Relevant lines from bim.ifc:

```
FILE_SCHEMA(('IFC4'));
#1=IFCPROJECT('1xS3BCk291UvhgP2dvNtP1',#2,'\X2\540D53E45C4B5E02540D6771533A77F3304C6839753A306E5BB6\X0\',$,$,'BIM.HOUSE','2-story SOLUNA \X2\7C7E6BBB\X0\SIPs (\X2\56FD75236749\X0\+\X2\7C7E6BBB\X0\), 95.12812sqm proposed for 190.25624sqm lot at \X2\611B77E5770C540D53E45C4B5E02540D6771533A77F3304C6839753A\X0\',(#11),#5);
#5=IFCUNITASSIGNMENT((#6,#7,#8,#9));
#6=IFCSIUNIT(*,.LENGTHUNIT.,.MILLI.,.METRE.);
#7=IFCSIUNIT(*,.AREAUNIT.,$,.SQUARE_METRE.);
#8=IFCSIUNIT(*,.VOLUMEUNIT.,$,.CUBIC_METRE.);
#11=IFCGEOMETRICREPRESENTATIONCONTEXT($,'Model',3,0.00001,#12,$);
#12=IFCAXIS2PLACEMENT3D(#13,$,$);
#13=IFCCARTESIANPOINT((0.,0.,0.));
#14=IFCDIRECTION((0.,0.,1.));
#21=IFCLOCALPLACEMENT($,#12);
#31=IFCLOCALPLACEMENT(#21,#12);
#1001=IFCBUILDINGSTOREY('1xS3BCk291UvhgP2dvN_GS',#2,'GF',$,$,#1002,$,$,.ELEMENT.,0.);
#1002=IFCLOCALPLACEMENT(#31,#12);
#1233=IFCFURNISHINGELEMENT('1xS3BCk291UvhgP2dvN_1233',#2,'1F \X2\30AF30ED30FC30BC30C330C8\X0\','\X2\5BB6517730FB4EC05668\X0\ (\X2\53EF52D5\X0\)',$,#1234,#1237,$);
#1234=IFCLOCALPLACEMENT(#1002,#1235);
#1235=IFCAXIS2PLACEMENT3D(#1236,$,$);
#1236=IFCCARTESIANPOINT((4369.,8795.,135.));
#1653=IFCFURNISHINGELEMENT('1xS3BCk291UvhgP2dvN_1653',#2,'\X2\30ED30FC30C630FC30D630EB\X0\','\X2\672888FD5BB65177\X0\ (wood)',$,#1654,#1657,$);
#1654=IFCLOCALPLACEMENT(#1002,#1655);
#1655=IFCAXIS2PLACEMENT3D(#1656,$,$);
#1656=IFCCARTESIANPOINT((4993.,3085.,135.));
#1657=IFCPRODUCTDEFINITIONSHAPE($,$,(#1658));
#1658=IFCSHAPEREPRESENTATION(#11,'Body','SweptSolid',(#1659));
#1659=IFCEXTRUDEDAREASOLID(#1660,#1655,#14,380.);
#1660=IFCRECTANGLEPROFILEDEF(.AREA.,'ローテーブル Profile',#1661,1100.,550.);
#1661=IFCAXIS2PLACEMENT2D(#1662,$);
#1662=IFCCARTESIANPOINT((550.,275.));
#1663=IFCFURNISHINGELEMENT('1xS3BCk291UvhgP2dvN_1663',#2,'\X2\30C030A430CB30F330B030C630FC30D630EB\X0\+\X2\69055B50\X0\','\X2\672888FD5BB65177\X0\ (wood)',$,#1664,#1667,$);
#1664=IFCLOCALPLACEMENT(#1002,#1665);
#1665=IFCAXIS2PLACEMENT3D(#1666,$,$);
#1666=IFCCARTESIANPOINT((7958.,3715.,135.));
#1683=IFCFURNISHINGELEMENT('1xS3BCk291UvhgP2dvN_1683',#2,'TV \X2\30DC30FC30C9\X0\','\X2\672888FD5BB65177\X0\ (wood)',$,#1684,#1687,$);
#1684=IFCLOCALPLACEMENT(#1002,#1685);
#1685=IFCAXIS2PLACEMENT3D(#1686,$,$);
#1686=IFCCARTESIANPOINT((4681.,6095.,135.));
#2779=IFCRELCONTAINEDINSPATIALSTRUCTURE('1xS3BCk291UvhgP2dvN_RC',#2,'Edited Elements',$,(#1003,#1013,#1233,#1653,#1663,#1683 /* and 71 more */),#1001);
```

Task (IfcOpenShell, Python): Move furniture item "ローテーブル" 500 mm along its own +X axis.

```python
import ifcopenshell
import ifcopenshell.api.geometry
import ifcopenshell.util.placement
import ifcopenshell.util.unit

model = ifcopenshell.open("bim.ifc")
unit_scale = ifcopenshell.util.unit.calculate_unit_scale(model)

item = model.by_id(1653)
matrix = ifcopenshell.util.placement.get_local_placement(item.ObjectPlacement)
matrix[:3, 3] += matrix[:3, 0] * 0.5 / unit_scale
ifcopenshell.api.geometry.edit_object_placement(model, product=item, matrix=matrix, is_si=False)

print(ifcopenshell.util.placement.get_local_placement(item.ObjectPlacement).round(3) + 0.0)

model.write("bim_v2.ifc")
```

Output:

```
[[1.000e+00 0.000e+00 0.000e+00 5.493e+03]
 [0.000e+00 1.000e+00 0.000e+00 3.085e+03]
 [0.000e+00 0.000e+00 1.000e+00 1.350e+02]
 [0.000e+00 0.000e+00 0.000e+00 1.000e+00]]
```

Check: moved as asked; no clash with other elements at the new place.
